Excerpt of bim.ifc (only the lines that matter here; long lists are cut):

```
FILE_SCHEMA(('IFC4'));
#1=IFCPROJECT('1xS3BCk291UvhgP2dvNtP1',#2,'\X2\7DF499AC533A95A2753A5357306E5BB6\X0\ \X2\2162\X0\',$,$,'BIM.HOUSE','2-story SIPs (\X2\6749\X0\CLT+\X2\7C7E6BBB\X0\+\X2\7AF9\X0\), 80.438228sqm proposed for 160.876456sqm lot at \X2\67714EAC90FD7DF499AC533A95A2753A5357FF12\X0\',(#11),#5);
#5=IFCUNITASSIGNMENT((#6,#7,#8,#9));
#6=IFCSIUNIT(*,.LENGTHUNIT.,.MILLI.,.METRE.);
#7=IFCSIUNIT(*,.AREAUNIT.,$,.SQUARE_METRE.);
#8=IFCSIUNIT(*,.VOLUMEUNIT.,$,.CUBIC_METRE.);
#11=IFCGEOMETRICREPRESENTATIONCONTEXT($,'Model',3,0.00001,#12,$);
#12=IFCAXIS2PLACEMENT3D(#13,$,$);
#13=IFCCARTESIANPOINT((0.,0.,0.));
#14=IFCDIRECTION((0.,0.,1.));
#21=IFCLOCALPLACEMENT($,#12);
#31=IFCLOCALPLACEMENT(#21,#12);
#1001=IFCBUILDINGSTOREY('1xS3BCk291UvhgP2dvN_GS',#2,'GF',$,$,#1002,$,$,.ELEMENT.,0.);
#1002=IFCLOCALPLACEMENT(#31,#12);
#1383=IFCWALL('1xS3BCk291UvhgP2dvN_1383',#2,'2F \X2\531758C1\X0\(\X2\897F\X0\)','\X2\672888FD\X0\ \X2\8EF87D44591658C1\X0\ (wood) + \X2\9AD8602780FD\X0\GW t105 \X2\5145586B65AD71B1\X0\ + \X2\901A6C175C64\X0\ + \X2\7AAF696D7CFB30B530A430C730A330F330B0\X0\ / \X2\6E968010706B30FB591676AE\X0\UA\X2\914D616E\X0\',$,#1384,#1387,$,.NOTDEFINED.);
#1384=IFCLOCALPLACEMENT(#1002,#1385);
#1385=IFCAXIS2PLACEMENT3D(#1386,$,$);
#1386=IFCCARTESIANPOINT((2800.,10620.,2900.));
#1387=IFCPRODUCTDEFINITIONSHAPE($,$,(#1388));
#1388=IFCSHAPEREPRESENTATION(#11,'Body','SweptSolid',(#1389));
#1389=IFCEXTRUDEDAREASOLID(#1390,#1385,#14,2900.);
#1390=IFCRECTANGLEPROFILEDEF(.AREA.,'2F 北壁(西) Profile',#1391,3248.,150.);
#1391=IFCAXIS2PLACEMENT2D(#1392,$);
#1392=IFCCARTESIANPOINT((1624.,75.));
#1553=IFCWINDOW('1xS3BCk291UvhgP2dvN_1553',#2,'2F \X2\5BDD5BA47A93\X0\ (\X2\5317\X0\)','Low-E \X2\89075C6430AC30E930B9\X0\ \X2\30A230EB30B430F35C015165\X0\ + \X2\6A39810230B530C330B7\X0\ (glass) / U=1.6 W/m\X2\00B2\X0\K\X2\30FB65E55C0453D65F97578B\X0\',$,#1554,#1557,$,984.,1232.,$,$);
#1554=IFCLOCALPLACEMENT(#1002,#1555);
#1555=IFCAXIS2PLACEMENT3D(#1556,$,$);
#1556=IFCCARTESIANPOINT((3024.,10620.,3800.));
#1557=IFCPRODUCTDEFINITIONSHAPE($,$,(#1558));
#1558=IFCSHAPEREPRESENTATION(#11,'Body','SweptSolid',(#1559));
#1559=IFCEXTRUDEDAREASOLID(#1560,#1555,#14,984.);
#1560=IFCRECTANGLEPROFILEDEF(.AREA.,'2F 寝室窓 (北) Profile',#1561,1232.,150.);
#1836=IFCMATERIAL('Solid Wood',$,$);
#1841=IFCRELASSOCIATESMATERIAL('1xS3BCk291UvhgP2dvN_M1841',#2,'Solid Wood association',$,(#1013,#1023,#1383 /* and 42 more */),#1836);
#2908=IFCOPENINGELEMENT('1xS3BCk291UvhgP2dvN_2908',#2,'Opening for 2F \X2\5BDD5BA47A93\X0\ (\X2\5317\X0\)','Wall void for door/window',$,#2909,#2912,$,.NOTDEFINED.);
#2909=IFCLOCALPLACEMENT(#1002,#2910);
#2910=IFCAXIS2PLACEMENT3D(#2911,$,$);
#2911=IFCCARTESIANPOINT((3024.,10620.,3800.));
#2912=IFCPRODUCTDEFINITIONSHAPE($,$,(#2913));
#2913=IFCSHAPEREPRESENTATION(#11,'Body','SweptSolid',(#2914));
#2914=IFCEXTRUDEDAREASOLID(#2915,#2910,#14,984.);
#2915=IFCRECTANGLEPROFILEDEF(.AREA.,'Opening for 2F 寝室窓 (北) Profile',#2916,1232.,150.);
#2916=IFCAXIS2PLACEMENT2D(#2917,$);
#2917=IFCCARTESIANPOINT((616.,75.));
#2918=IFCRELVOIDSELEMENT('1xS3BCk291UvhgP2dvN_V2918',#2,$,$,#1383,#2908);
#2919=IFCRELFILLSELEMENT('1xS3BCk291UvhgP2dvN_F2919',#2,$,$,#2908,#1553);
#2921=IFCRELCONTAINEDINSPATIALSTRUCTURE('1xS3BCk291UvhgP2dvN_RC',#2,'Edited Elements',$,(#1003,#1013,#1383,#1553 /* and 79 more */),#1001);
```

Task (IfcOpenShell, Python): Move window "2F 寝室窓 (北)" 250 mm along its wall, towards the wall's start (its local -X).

```python
import ifcopenshell
import ifcopenshell.api.geometry
import ifcopenshell.util.placement

model = ifcopenshell.open("bim.ifc")

window = model.by_id(1553)
opening = window.FillsVoids[0].RelatingOpeningElement
wall = opening.VoidsElements[0].RelatingBuildingElement

wall_matrix = ifcopenshell.util.placement.get_local_placement(wall.ObjectPlacement)
shift = wall_matrix[:3, 0] * -250.0
before = ifcopenshell.util.placement.get_local_placement(window.ObjectPlacement)[:3, 3].copy()

# The window is not placed relative to its opening, so move both.
for product in (opening, window):
    matrix = ifcopenshell.util.placement.get_local_placement(product.ObjectPlacement)
    matrix[:3, 3] += shift
    ifcopenshell.api.geometry.edit_object_placement(model, product=product, matrix=matrix, is_si=False)

after = ifcopenshell.util.placement.get_local_placement(window.ObjectPlacement)[:3, 3]
print("window moved by", (after - before).round(3) + 0.0)

model.write("bim_rev.ifc")
```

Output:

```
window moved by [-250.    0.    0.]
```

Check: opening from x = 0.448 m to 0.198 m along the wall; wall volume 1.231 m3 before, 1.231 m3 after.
